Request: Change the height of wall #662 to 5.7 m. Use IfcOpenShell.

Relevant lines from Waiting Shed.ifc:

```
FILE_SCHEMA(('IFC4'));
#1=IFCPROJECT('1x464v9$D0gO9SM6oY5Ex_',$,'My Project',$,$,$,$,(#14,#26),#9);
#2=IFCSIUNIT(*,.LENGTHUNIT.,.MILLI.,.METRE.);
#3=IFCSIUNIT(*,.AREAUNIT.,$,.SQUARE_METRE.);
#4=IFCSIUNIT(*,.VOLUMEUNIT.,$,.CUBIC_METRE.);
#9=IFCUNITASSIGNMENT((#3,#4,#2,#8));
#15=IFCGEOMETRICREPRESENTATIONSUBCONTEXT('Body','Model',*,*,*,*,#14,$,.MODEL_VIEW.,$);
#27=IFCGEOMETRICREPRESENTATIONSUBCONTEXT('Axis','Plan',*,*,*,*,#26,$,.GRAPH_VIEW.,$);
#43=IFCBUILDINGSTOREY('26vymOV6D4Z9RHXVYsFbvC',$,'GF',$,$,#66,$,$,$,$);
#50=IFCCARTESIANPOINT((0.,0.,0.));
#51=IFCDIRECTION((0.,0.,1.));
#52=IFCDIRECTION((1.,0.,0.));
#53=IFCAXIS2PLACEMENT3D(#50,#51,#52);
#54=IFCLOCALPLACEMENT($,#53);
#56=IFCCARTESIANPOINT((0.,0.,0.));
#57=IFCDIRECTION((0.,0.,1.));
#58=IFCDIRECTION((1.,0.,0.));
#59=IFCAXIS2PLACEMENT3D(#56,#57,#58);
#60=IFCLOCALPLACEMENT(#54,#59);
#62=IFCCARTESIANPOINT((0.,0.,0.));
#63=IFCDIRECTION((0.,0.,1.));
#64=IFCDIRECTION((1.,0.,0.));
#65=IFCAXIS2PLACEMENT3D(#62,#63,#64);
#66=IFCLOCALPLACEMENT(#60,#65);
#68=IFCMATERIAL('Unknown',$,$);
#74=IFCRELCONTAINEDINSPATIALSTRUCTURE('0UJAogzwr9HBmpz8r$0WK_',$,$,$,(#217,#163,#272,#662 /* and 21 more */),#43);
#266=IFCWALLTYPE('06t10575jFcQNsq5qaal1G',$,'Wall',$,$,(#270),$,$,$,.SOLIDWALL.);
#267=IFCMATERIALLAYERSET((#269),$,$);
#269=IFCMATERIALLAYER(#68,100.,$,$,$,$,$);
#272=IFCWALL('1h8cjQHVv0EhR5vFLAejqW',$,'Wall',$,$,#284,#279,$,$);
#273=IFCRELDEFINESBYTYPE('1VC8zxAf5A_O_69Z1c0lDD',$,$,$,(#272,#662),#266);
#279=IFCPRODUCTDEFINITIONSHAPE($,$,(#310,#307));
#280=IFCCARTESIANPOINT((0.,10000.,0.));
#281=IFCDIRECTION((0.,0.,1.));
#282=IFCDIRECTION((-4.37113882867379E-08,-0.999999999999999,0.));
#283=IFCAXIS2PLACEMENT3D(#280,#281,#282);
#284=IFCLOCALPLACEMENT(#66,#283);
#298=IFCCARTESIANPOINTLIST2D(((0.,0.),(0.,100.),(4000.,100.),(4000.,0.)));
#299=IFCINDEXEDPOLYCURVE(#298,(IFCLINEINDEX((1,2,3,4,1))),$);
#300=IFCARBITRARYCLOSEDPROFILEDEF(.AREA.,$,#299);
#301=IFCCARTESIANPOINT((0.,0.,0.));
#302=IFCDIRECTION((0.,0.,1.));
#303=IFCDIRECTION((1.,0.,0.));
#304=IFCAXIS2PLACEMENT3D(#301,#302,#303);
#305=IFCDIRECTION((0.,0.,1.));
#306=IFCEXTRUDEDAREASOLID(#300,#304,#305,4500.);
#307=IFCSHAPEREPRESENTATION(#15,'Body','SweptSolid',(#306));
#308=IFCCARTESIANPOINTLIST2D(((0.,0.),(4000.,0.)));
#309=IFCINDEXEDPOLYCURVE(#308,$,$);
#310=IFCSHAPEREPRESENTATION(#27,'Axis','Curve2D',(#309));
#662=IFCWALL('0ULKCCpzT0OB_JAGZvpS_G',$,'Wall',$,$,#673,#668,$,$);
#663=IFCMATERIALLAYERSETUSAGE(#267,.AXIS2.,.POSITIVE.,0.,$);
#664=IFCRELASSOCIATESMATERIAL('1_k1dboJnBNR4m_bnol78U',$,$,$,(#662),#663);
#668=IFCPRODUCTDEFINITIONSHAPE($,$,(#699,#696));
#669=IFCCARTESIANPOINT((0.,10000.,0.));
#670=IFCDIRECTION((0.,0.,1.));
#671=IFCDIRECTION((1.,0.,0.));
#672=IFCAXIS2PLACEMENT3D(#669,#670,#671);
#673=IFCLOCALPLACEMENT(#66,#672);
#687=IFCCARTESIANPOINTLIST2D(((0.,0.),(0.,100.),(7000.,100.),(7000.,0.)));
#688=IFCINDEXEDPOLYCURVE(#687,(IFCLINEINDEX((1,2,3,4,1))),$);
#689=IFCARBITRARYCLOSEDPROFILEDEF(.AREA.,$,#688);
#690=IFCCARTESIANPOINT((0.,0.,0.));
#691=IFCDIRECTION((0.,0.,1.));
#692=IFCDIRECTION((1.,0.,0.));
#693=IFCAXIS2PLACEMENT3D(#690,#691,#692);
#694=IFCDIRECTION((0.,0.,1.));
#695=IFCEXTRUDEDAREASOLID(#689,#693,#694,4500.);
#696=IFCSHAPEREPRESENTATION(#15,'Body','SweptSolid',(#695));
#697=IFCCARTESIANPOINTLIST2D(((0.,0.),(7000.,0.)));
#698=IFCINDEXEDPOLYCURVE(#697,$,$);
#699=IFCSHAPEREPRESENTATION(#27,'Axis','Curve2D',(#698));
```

```python
import ifcopenshell
import ifcopenshell.geom
import ifcopenshell.util.representation
import ifcopenshell.util.shape
import ifcopenshell.util.unit

model = ifcopenshell.open("Waiting Shed.ifc")
unit_scale = ifcopenshell.util.unit.calculate_unit_scale(model)
settings = ifcopenshell.geom.settings()


def volume(element):
    """Net volume in cubic metres, openings subtracted."""
    shape = ifcopenshell.geom.create_shape(settings, element)
    return ifcopenshell.util.shape.get_volume(shape.geometry)


wall = model.by_id(662)
before = volume(wall)

body = ifcopenshell.util.representation.get_representation(wall, "Model", "Body")
solid = body.Items[0]
old_height = solid.Depth
solid.Depth = 5.7 / unit_scale
after = volume(wall)

print(f"height {old_height:g} -> {solid.Depth:g}, volume {before:.3f} -> {after:.3f} m3")

model.write("Waiting Shed-out.ifc")
```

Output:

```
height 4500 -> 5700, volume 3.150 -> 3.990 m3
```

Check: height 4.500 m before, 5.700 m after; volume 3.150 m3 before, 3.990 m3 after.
